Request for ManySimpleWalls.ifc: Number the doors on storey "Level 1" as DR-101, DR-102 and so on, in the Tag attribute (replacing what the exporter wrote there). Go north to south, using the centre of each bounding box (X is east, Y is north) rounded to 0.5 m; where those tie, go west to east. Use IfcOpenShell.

First a look at what the model holds.

```python
import ifcopenshell
import ifcopenshell.util.element
import ifcopenshell.util.placement

model = ifcopenshell.open("ManySimpleWalls.ifc")
print(model.schema)
storey = next(s for s in model.by_type("IfcBuildingStorey") if s.Name == "Level 1")
doors = [e for e in ifcopenshell.util.element.get_decomposition(storey) if e.is_a("IfcDoor")]
for e in sorted(doors, key=lambda e: e.id()):
    origin = ifcopenshell.util.placement.get_local_placement(e.ObjectPlacement)[:3, 3]
    print(e.id(), e.Tag, e.Name, origin.round(2) + 0.0, sep=" | ")
```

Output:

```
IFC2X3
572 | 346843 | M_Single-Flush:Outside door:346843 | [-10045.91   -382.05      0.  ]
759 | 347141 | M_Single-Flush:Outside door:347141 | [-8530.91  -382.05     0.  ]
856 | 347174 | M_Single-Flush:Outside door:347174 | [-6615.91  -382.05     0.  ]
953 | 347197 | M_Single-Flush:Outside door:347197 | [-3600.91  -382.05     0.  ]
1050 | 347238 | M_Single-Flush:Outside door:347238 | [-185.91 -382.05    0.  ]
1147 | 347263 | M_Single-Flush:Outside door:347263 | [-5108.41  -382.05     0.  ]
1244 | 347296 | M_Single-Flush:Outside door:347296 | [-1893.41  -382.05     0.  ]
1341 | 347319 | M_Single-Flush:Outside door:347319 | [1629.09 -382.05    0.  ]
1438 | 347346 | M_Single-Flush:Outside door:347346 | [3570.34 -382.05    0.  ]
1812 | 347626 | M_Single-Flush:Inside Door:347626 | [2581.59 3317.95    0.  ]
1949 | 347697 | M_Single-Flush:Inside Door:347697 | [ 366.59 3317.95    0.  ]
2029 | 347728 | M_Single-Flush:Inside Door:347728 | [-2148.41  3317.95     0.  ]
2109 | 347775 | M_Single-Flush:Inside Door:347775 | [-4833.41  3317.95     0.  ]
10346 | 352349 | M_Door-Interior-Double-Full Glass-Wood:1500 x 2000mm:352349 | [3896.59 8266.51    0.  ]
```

```python
import ifcopenshell
import ifcopenshell.geom
import ifcopenshell.util.element
import ifcopenshell.util.shape

model = ifcopenshell.open("ManySimpleWalls.ifc")
settings = ifcopenshell.geom.settings()
settings.set("use-world-coords", True)


def centre(element):
    shape = ifcopenshell.geom.create_shape(settings, element)
    return ifcopenshell.util.shape.get_bbox_centroid(shape.geometry)


storey = next(s for s in model.by_type("IfcBuildingStorey") if s.Name == "Level 1")
doors = [e for e in ifcopenshell.util.element.get_decomposition(storey) if e.is_a("IfcDoor")]

# Insertion points can sit at a corner or the storey origin, so sort by the geometry (in metres).
centres = {e: centre(e) for e in doors}
doors.sort(key=lambda e: (-round(centres[e][1] / 0.5), centres[e][0]))

for i, e in enumerate(doors, start=1):
    number = f"DR-1{i:02d}"
    e.Tag = number
    print(e.id(), number)

model.write("ManySimpleWalls-out.ifc")
```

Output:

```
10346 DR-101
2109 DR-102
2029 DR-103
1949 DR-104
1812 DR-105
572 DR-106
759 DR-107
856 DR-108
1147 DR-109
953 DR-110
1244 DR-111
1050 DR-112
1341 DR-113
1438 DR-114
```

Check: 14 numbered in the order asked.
